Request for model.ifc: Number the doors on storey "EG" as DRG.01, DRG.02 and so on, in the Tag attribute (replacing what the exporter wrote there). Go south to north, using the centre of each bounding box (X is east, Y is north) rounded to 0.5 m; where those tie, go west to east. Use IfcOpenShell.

First a look at what the model holds.

```python
import ifcopenshell
import ifcopenshell.util.element
import ifcopenshell.util.placement

model = ifcopenshell.open("model.ifc")
print(model.schema)
storey = next(s for s in model.by_type("IfcBuildingStorey") if s.Name == "EG")
doors = [e for e in ifcopenshell.util.element.get_decomposition(storey) if e.is_a("IfcDoor")]
for e in sorted(doors, key=lambda e: e.id()):
    origin = ifcopenshell.util.placement.get_local_placement(e.ObjectPlacement)[:3, 3]
    print(e.id(), e.Tag, e.Name, origin.round(2) + 0.0, sep=" | ")
```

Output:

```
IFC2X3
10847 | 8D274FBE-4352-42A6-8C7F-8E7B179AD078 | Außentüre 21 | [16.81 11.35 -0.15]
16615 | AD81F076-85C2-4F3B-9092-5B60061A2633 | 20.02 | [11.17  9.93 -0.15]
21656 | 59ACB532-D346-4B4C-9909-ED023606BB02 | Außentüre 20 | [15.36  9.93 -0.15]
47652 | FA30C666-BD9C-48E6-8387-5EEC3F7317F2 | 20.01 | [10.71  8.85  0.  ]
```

```python
import ifcopenshell
import ifcopenshell.geom
import ifcopenshell.util.element
import ifcopenshell.util.shape

model = ifcopenshell.open("model.ifc")
settings = ifcopenshell.geom.settings()
settings.set("use-world-coords", True)


def centre(element):
    shape = ifcopenshell.geom.create_shape(settings, element)
    return ifcopenshell.util.shape.get_bbox_centroid(shape.geometry)


storey = next(s for s in model.by_type("IfcBuildingStorey") if s.Name == "EG")
doors = [e for e in ifcopenshell.util.element.get_decomposition(storey) if e.is_a("IfcDoor")]

# Insertion points can sit at a corner or the storey origin, so sort by the geometry (in metres).
centres = {e: centre(e) for e in doors}
doors.sort(key=lambda e: (round(centres[e][1] / 0.5), centres[e][0]))

for i, e in enumerate(doors, start=1):
    number = f"DRG.{i:02d}"
    e.Tag = number
    print(e.id(), number)

model.write("model-out.ifc")
```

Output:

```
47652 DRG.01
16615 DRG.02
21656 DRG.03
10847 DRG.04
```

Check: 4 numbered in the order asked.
